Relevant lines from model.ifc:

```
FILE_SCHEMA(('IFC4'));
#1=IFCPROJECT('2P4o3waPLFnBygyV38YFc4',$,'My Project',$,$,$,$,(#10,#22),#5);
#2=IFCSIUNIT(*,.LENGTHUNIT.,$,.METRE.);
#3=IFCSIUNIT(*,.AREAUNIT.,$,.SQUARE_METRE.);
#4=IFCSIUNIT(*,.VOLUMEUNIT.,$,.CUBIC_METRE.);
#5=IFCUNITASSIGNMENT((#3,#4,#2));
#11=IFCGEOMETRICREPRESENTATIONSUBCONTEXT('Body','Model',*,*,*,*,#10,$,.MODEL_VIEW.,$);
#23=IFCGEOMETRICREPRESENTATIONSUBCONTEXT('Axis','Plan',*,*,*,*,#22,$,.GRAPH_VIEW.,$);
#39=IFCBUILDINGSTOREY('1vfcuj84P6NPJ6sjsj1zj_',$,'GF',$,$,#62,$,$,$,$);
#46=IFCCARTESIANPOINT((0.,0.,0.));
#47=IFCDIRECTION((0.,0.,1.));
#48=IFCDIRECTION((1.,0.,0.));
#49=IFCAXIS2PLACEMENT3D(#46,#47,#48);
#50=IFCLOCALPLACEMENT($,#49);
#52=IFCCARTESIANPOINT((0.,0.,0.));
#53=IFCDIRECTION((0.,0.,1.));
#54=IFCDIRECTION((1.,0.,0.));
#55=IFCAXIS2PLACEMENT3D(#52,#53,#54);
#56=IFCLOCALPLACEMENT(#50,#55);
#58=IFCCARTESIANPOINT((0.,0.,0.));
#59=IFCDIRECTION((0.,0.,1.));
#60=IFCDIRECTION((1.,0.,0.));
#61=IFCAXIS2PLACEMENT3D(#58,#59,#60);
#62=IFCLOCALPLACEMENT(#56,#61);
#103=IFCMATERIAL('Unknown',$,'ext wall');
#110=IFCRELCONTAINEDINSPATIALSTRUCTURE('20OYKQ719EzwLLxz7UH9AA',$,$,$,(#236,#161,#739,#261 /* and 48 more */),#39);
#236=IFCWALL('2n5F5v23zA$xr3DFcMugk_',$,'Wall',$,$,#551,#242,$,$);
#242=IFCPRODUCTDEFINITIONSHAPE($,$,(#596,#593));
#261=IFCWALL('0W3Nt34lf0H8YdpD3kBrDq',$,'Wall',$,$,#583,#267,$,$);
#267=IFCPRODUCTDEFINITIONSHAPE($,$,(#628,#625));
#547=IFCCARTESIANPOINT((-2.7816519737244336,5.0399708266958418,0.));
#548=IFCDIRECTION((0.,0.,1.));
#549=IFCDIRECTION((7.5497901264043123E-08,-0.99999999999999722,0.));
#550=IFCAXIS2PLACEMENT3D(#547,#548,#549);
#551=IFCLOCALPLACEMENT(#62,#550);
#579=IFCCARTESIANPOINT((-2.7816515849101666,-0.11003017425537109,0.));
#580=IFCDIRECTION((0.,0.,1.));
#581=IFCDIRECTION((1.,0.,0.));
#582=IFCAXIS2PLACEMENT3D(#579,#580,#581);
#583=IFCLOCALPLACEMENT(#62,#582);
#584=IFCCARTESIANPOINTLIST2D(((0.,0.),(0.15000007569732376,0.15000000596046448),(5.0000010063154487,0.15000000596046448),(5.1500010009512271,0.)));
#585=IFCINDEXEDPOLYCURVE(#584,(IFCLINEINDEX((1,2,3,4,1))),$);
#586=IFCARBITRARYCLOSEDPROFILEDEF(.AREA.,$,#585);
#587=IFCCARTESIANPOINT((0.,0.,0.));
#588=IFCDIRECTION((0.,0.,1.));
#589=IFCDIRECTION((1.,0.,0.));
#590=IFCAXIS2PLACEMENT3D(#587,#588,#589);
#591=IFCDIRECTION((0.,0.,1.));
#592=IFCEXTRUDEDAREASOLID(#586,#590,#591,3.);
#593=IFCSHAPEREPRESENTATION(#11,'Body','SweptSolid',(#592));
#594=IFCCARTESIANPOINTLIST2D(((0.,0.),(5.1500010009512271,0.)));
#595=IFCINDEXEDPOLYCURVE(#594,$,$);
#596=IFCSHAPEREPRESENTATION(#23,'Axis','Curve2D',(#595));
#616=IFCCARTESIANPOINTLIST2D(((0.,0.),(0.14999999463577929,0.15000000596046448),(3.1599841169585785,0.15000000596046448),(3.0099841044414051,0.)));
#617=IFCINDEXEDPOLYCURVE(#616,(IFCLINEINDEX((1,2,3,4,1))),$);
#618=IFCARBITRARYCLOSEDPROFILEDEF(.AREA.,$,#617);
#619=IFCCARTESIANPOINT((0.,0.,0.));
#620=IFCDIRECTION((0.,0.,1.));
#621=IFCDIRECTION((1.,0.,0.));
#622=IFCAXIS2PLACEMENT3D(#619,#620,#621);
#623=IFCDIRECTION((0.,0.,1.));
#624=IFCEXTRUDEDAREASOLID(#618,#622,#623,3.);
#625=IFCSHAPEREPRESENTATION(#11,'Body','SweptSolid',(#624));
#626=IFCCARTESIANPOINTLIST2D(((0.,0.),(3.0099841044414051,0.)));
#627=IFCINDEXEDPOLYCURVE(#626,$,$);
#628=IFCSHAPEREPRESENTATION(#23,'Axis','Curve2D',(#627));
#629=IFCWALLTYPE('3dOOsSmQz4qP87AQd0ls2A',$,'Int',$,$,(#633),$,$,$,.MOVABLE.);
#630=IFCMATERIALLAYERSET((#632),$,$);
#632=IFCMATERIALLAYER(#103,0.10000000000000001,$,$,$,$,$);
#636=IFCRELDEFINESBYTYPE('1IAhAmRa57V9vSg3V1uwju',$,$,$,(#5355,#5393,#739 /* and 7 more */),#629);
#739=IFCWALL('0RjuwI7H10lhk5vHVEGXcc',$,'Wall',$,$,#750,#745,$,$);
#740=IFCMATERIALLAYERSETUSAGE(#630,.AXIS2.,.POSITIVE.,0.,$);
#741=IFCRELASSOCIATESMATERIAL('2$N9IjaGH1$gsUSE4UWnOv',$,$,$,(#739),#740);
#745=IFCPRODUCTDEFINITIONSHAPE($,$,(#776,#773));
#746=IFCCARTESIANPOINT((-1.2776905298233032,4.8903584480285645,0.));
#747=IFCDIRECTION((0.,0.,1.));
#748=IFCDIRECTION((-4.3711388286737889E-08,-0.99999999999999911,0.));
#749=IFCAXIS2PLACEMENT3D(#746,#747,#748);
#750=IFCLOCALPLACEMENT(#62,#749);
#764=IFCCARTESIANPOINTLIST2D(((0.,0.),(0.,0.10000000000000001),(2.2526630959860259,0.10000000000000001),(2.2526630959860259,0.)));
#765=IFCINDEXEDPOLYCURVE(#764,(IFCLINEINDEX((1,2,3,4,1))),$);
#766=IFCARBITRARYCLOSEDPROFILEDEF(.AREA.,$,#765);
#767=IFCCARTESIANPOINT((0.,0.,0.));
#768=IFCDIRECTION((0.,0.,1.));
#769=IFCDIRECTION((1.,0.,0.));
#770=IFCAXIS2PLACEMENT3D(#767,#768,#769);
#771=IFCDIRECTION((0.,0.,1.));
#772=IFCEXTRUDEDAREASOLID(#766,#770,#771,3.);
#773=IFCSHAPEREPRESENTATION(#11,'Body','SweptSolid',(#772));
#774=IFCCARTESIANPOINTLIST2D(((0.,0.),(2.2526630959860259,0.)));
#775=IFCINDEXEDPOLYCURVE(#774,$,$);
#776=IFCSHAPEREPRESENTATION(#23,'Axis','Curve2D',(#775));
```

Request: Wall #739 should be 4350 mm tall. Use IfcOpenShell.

```python
import ifcopenshell
import ifcopenshell.geom
import ifcopenshell.util.representation
import ifcopenshell.util.shape

model = ifcopenshell.open("model.ifc")
settings = ifcopenshell.geom.settings()


def volume(element):
    """Net volume in cubic metres, openings subtracted."""
    shape = ifcopenshell.geom.create_shape(settings, element)
    return ifcopenshell.util.shape.get_volume(shape.geometry)


wall = model.by_guid("0RjuwI7H10lhk5vHVEGXcc")
before = volume(wall)

body = ifcopenshell.util.representation.get_representation(wall, "Model", "Body")
solid = body.Items[0]
old_height = solid.Depth
solid.Depth = 4.35
after = volume(wall)

print(f"height {old_height:g} -> {solid.Depth:g}, volume {before:.3f} -> {after:.3f} m3")

model.write("model_rev.ifc")
```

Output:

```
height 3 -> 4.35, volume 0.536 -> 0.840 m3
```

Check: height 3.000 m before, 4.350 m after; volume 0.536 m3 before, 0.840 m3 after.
